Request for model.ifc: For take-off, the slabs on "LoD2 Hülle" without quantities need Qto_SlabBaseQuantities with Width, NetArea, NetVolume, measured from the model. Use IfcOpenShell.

First a look at what the model holds.

```python
import ifcopenshell
import ifcopenshell.util.element
import ifcopenshell.util.unit

model = ifcopenshell.open("model.ifc")
print(model.schema)
for unit_type in ("LENGTHUNIT", "AREAUNIT", "VOLUMEUNIT"):
    print(unit_type, ifcopenshell.util.unit.calculate_unit_scale(model, unit_type))
storey = next(s for s in model.by_type("IfcBuildingStorey") if s.Name == "LoD2 Hülle")
slabs = [e for e in ifcopenshell.util.element.get_decomposition(storey) if e.is_a("IfcSlab")]
for e in sorted(slabs, key=lambda e: e.id()):
    print(e.id(), e.is_a(), e.Name, list(ifcopenshell.util.element.get_psets(e, qtos_only=True)), sep=" | ")
```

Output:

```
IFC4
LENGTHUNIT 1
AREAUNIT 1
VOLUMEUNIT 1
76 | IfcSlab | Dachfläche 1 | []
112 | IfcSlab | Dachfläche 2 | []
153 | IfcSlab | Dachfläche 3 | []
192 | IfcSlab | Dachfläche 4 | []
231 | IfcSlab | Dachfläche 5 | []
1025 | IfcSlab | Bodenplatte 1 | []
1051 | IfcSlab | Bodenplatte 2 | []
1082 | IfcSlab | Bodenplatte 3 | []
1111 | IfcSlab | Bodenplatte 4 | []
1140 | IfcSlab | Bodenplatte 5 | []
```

```python
import ifcopenshell
import ifcopenshell.api.pset
import ifcopenshell.geom
import ifcopenshell.util.element
import ifcopenshell.util.shape
import ifcopenshell.util.unit

model = ifcopenshell.open("model.ifc")
unit_scale = ifcopenshell.util.unit.calculate_unit_scale(model)
area_scale = ifcopenshell.util.unit.calculate_unit_scale(model, "AREAUNIT")
volume_scale = ifcopenshell.util.unit.calculate_unit_scale(model, "VOLUMEUNIT")
settings = ifcopenshell.geom.settings()

storey = next(s for s in model.by_type("IfcBuildingStorey") if s.Name == "LoD2 Hülle")
slabs = [e for e in ifcopenshell.util.element.get_decomposition(storey) if e.is_a("IfcSlab")]

for e in sorted(slabs, key=lambda e: e.id()):
    if ifcopenshell.util.element.get_psets(e, qtos_only=True, should_inherit=False):
        continue
    # Geometry comes back in metres, in the element's own axes.
    shape = ifcopenshell.geom.create_shape(settings, e)
    values = {
        "Width": ifcopenshell.util.shape.get_z(shape.geometry) / unit_scale,
        "NetArea": ifcopenshell.util.shape.get_footprint_area(shape.geometry) / area_scale,
        "NetVolume": ifcopenshell.util.shape.get_volume(shape.geometry) / volume_scale,
    }
    qto = ifcopenshell.api.pset.add_qto(model, product=e, name="Qto_SlabBaseQuantities")
    ifcopenshell.api.pset.edit_qto(model, qto=qto, properties=values)
    print(e.id(), {k: round(v, 3) for k, v in values.items()})

model.write("model-out.ifc")
```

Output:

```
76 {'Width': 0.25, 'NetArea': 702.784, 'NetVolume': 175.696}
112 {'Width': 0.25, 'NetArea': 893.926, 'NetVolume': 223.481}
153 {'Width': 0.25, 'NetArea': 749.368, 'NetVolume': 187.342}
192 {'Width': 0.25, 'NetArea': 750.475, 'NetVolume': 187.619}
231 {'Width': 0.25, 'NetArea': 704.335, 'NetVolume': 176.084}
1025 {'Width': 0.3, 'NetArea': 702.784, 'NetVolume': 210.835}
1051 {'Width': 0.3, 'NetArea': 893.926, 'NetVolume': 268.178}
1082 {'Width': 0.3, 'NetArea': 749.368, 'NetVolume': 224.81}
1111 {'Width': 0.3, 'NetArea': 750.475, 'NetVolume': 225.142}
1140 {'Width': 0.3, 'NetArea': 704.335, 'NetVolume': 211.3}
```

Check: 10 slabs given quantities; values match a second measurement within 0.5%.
